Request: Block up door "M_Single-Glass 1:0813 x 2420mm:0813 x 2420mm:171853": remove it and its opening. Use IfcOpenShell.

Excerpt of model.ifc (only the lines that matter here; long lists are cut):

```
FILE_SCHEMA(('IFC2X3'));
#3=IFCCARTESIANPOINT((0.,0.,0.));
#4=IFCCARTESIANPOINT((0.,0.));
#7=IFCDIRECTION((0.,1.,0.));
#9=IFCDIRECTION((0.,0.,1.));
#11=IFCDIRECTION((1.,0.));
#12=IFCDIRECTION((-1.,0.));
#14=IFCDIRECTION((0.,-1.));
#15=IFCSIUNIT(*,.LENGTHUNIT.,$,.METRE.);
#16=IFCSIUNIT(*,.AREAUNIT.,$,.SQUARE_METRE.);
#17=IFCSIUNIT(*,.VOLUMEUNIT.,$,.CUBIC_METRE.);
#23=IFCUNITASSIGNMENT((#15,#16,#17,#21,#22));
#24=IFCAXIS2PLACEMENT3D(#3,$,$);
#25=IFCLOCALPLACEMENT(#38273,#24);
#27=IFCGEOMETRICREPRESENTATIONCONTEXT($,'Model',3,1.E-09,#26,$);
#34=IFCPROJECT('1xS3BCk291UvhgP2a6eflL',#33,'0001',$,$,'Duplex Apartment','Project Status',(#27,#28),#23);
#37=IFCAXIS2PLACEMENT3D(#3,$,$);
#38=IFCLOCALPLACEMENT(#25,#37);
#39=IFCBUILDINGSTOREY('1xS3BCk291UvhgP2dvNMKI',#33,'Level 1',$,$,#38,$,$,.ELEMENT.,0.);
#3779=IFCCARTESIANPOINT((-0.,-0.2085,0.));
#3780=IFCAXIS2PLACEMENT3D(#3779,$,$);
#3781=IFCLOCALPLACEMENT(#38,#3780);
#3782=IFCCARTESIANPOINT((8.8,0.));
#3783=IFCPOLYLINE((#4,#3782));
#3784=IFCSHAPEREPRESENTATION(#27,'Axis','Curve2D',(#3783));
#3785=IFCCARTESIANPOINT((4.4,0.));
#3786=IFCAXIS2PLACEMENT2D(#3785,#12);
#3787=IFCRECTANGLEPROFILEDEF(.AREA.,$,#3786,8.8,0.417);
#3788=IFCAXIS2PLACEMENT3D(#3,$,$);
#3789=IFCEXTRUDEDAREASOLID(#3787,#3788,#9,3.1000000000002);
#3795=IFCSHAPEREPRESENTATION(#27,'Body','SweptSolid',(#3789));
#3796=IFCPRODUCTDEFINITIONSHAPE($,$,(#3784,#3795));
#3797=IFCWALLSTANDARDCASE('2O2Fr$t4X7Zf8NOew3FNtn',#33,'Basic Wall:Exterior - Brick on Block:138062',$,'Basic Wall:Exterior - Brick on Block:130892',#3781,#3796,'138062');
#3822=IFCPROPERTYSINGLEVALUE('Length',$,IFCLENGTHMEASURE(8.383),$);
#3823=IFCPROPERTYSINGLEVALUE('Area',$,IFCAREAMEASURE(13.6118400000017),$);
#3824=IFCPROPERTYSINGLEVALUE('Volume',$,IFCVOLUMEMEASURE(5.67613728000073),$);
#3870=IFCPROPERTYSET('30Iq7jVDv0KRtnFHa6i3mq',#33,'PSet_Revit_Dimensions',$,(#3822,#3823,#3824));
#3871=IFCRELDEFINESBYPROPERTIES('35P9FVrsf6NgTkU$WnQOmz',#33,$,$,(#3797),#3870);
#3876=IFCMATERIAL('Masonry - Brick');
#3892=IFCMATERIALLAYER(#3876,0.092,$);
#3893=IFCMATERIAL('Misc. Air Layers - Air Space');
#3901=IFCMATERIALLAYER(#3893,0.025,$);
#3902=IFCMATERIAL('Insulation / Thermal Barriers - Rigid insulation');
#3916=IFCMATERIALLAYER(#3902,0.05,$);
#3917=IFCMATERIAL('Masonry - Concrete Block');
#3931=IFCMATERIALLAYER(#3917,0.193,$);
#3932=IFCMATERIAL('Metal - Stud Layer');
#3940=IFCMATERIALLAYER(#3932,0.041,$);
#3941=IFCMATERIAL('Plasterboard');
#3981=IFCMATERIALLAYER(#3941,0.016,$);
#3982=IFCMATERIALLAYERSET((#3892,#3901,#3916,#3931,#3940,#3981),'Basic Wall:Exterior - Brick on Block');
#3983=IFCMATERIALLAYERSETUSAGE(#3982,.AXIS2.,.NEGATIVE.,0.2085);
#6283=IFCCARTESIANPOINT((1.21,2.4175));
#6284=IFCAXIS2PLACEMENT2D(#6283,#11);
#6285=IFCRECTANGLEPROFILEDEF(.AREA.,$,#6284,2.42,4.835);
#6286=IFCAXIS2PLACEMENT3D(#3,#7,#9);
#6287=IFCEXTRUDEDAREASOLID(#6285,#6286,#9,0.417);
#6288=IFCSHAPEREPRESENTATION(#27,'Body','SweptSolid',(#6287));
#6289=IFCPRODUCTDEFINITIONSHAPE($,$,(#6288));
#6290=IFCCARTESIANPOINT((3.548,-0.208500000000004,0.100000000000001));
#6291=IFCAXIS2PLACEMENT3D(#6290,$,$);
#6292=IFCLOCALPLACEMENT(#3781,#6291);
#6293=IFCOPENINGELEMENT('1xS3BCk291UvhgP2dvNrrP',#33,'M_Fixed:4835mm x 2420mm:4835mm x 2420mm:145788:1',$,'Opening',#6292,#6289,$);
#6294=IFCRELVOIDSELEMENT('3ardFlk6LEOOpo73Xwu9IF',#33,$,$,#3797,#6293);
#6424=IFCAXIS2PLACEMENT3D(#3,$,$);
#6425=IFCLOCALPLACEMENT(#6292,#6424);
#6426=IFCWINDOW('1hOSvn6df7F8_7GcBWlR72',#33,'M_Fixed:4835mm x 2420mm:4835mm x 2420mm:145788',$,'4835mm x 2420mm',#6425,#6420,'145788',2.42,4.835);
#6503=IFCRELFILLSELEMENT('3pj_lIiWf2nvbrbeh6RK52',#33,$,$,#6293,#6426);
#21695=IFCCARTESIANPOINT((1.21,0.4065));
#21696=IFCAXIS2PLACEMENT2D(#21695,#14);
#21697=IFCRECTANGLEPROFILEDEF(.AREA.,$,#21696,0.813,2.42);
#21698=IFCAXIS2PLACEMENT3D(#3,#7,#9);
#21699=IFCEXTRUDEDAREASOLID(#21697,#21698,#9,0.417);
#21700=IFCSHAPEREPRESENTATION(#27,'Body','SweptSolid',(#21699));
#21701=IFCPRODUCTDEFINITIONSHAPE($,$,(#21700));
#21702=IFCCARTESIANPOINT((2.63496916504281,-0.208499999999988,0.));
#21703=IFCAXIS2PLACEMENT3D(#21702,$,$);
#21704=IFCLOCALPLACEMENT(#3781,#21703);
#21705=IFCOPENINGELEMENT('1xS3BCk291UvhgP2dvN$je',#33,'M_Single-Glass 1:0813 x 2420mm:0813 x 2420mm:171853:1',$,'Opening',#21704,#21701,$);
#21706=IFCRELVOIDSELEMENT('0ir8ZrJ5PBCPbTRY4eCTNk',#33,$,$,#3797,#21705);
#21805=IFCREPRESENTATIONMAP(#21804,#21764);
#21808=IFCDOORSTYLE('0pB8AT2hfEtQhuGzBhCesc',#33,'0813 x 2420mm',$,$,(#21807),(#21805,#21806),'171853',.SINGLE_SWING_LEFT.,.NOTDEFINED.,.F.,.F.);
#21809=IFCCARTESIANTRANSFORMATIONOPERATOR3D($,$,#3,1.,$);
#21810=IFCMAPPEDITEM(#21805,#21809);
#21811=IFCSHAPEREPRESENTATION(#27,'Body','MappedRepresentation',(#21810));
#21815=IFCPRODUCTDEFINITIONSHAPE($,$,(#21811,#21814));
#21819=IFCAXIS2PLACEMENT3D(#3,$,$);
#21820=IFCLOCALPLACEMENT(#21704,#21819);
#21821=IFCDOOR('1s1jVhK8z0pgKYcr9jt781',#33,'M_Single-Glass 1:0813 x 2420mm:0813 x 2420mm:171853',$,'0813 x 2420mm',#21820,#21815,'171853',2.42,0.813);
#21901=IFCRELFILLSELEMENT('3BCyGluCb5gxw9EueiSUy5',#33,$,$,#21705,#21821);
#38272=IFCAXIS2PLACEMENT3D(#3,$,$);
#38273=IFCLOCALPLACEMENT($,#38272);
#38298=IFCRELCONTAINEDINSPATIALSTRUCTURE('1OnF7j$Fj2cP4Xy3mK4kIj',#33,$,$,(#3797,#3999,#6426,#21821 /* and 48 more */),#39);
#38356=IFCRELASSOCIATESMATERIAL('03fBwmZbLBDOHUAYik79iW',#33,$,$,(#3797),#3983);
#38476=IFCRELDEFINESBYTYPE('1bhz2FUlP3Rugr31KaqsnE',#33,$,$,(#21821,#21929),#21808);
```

```python
import ifcopenshell
import ifcopenshell.api.feature
import ifcopenshell.api.pset
import ifcopenshell.api.root
import ifcopenshell.geom
import ifcopenshell.util.element
import ifcopenshell.util.shape
import ifcopenshell.util.unit

model = ifcopenshell.open("model.ifc")
area_scale = ifcopenshell.util.unit.calculate_unit_scale(model, "AREAUNIT")
volume_scale = ifcopenshell.util.unit.calculate_unit_scale(model, "VOLUMEUNIT")
settings = ifcopenshell.geom.settings()


def volume(element):
    """Net volume in cubic metres, openings subtracted."""
    shape = ifcopenshell.geom.create_shape(settings, element)
    return ifcopenshell.util.shape.get_volume(shape.geometry)


door = model.by_guid("1s1jVhK8z0pgKYcr9jt781")
opening = door.FillsVoids[0].RelatingOpeningElement
wall = opening.VoidsElements[0].RelatingBuildingElement
before = volume(wall)

ifcopenshell.api.root.remove_product(model, product=door)
ifcopenshell.api.feature.remove_feature(model, feature=opening)

after = volume(wall)
thickness = 0.417  # wall thickness in metres

# Update the wall's stored quantities.
pset = model.by_id(ifcopenshell.util.element.get_pset(wall, "PSet_Revit_Dimensions", should_inherit=False)["id"])
ifcopenshell.api.pset.edit_pset(model, pset=pset, properties={
    "Area": model.create_entity("IfcAreaMeasure", after / thickness / area_scale),
    "Volume": model.create_entity("IfcVolumeMeasure", after / volume_scale),
})

print(f"wall volume {before:.3f} -> {after:.3f} m3")

model.write("model_v2.ifc")
```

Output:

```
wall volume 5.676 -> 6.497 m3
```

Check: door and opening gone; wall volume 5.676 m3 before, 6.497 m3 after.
